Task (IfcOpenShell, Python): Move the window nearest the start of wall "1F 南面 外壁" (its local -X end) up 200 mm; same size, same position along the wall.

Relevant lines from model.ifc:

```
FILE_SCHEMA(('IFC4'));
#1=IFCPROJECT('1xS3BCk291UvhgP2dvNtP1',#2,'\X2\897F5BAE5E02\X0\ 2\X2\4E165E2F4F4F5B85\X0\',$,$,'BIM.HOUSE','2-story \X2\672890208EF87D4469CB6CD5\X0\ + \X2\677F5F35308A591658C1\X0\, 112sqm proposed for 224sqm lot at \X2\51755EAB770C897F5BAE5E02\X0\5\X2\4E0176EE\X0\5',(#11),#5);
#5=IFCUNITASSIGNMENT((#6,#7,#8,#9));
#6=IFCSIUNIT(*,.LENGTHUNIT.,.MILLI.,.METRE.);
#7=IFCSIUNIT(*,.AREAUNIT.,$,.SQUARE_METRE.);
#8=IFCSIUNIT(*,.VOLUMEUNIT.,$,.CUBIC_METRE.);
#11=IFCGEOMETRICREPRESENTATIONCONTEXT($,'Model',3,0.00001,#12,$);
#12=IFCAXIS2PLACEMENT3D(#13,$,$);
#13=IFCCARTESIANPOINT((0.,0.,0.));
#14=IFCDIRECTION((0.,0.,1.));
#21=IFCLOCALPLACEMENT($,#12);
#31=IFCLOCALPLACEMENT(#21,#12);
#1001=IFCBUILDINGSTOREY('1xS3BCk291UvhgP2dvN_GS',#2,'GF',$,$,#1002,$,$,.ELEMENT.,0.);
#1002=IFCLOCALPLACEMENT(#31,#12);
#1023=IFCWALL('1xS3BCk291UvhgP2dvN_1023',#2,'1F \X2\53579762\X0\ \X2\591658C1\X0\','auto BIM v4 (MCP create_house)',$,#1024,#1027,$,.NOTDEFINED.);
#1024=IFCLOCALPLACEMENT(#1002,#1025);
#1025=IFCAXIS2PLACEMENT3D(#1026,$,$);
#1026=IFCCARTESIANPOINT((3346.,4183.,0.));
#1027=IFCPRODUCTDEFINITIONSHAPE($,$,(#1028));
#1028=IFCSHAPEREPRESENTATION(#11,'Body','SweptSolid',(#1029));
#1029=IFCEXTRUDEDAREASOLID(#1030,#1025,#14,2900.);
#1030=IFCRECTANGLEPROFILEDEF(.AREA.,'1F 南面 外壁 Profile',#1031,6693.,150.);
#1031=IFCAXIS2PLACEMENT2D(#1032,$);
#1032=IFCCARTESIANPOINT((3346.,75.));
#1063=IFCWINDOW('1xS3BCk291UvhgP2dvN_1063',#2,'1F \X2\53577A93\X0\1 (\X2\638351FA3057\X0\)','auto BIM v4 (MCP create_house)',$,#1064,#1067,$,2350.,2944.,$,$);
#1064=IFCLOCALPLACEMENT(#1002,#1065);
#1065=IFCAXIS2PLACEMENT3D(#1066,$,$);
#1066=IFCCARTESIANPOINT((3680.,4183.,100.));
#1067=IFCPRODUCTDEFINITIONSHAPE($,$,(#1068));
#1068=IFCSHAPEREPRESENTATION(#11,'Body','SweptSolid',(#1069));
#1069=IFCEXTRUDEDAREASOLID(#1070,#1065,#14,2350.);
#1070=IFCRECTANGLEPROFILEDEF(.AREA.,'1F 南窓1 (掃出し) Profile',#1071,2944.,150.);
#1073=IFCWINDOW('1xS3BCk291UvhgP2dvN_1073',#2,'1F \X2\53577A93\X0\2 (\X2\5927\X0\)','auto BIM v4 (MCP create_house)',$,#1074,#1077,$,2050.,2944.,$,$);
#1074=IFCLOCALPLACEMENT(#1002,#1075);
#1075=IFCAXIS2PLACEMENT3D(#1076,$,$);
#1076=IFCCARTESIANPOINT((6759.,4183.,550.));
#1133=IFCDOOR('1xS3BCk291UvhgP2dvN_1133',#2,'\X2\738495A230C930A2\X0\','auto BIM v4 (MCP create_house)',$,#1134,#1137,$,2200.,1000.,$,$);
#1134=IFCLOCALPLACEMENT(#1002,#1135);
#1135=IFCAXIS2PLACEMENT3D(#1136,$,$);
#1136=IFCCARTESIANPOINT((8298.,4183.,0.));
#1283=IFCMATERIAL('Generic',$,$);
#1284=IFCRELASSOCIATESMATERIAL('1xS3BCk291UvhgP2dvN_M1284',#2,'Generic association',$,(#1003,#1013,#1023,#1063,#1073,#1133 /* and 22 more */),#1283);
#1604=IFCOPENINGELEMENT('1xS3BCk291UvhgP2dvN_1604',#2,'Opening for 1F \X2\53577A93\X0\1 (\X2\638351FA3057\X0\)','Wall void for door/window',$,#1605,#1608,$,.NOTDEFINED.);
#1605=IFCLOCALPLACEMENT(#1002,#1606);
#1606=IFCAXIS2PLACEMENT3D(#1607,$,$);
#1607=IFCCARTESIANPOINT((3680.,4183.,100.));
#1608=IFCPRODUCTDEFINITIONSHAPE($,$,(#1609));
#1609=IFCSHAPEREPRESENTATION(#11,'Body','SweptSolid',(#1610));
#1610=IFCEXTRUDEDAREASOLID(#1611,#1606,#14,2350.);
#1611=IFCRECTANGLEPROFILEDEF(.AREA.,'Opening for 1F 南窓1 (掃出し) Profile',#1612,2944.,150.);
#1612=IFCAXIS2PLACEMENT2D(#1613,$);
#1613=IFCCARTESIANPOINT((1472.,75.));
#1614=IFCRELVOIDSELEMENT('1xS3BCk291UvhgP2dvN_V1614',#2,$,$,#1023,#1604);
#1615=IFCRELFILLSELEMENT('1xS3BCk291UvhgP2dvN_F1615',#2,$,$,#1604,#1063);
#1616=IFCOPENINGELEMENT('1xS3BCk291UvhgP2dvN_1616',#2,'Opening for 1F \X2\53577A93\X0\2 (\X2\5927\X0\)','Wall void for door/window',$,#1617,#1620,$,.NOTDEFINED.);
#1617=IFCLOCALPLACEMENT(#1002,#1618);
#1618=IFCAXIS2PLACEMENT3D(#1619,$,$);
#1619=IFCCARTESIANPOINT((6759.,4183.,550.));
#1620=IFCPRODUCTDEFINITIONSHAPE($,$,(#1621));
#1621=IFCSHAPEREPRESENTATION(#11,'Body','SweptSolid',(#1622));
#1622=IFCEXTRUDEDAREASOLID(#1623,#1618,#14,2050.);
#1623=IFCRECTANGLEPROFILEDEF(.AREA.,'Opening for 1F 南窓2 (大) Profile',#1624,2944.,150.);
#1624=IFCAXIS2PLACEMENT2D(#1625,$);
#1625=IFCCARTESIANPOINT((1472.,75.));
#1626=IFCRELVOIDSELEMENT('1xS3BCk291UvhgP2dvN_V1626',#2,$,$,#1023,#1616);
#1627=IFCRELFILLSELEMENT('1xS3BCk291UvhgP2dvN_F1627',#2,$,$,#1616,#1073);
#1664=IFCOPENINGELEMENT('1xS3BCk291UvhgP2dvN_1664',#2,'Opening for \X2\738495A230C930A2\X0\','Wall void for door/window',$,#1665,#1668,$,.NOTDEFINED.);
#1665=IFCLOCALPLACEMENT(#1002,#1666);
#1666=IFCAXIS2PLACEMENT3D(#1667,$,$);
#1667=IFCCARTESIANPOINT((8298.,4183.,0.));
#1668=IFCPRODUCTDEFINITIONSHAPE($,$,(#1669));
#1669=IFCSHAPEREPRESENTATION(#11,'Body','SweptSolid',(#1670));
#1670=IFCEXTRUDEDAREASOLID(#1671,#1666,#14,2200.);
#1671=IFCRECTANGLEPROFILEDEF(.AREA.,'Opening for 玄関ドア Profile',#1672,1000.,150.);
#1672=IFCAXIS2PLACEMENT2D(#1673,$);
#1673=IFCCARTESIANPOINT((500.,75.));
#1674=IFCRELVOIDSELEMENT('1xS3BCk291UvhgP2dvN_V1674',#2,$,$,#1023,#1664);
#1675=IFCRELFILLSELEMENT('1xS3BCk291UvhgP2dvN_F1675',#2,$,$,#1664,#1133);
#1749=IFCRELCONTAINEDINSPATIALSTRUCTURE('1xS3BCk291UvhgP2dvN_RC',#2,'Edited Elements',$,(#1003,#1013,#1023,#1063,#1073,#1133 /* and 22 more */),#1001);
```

```python
import numpy as np
import ifcopenshell
import ifcopenshell.api.geometry
import ifcopenshell.util.placement
import ifcopenshell.util.unit

model = ifcopenshell.open("model.ifc")
unit_scale = ifcopenshell.util.unit.calculate_unit_scale(model)

window = model.by_guid("1xS3BCk291UvhgP2dvN_1063")
opening = window.FillsVoids[0].RelatingOpeningElement
dz = 0.2 / unit_scale

shift = np.array([0.0, 0.0, dz])
# The window is not placed relative to its opening, so move both.
for product in (opening, window):
    matrix = ifcopenshell.util.placement.get_local_placement(product.ObjectPlacement)
    matrix[:3, 3] += shift
    ifcopenshell.api.geometry.edit_object_placement(model, product=product, matrix=matrix, is_si=False)

print(f"moved by {dz * unit_scale:+.3f} m")

model.write("model_updated.ifc")
```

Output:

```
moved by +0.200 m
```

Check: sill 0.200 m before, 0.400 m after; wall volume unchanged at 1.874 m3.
